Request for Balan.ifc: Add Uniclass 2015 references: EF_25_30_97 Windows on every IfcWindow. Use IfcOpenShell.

First a look at what the model holds.

```python
import ifcopenshell

model = ifcopenshell.open("Balan.ifc")
print(model.schema)
print("classifications:", [c.Name for c in model.by_type("IfcClassification")])
for ifc_class in ("IfcDoor", "IfcRoof", "IfcStair", "IfcWall", "IfcWindow"):
    print(ifc_class, len(model.by_type(ifc_class)))
```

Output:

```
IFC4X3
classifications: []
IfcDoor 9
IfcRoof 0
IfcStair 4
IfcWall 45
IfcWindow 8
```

```python
import ifcopenshell
import ifcopenshell.api.classification

model = ifcopenshell.open("Balan.ifc")

system = ifcopenshell.api.classification.add_classification(model, classification="Uniclass 2015")

codes = {
    "IfcWindow": ("EF_25_30_97", "Windows"),
}
for ifc_class, (code, name) in codes.items():
    products = model.by_type(ifc_class)
    ifcopenshell.api.classification.add_reference(
        model, products=products, classification=system, identification=code, name=name
    )
    print(code, len(products))

model.write("Balan_edited.ifc")
```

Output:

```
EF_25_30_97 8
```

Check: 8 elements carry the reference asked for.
